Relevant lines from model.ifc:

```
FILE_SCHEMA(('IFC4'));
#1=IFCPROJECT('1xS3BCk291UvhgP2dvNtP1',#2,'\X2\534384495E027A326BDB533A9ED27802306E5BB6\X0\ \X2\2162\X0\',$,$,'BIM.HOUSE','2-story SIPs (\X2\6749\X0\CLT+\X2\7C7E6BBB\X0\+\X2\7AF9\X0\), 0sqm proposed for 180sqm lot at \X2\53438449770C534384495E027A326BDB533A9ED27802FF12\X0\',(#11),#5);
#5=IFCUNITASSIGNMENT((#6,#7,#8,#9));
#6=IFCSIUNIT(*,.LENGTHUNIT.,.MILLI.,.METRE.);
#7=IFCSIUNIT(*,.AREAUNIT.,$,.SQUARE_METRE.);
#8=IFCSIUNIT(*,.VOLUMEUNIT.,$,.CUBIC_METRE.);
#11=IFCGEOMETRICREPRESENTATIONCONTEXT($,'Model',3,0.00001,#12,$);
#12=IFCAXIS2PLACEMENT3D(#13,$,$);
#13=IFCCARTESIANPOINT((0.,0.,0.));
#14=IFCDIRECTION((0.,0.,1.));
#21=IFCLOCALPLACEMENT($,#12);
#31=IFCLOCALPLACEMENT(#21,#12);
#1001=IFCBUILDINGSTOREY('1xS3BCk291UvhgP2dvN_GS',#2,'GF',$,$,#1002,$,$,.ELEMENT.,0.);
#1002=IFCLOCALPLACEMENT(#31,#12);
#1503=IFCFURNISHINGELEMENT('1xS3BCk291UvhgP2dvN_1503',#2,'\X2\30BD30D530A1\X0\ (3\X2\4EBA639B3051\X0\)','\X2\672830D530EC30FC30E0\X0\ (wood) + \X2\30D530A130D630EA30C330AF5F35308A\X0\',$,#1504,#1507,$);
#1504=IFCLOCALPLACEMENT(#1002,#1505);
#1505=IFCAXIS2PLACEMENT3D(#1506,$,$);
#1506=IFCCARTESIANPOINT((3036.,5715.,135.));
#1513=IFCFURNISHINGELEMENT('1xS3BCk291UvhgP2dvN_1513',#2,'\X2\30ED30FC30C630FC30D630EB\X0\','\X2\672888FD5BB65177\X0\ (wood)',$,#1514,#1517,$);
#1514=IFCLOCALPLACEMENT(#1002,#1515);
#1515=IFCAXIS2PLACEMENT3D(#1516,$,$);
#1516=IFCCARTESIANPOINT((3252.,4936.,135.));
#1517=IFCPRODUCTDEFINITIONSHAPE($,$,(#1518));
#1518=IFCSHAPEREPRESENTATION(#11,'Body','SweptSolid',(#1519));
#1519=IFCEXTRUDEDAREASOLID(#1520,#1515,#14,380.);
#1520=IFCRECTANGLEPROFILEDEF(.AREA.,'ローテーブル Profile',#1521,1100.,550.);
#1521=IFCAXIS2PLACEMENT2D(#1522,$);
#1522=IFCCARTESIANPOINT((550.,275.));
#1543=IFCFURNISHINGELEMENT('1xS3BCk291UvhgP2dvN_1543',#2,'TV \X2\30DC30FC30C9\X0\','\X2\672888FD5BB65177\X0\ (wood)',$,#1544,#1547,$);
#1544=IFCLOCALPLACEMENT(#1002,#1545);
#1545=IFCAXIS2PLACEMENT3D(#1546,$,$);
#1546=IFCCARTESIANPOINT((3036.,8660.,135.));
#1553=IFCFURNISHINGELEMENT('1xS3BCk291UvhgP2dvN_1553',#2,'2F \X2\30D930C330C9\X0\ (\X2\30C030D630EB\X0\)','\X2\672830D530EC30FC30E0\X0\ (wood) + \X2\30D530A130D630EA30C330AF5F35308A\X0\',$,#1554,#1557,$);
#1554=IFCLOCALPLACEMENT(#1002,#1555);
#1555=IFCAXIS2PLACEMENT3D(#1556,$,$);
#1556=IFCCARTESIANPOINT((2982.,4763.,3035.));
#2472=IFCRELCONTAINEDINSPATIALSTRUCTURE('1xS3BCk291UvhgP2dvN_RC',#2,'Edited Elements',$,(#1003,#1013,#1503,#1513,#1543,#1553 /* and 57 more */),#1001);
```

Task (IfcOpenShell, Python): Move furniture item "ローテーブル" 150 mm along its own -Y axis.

```python
import ifcopenshell
import ifcopenshell.api.geometry
import ifcopenshell.util.placement
import ifcopenshell.util.unit

model = ifcopenshell.open("model.ifc")
unit_scale = ifcopenshell.util.unit.calculate_unit_scale(model)

item = model.by_guid("1xS3BCk291UvhgP2dvN_1513")
matrix = ifcopenshell.util.placement.get_local_placement(item.ObjectPlacement)
matrix[:3, 3] -= matrix[:3, 1] * 0.15 / unit_scale
ifcopenshell.api.geometry.edit_object_placement(model, product=item, matrix=matrix, is_si=False)

print(ifcopenshell.util.placement.get_local_placement(item.ObjectPlacement).round(3) + 0.0)

model.write("model_rev.ifc")
```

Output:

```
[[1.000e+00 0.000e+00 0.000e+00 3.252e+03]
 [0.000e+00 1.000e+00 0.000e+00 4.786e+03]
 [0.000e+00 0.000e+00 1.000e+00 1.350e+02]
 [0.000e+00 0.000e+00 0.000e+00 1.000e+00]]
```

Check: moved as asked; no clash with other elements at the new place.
